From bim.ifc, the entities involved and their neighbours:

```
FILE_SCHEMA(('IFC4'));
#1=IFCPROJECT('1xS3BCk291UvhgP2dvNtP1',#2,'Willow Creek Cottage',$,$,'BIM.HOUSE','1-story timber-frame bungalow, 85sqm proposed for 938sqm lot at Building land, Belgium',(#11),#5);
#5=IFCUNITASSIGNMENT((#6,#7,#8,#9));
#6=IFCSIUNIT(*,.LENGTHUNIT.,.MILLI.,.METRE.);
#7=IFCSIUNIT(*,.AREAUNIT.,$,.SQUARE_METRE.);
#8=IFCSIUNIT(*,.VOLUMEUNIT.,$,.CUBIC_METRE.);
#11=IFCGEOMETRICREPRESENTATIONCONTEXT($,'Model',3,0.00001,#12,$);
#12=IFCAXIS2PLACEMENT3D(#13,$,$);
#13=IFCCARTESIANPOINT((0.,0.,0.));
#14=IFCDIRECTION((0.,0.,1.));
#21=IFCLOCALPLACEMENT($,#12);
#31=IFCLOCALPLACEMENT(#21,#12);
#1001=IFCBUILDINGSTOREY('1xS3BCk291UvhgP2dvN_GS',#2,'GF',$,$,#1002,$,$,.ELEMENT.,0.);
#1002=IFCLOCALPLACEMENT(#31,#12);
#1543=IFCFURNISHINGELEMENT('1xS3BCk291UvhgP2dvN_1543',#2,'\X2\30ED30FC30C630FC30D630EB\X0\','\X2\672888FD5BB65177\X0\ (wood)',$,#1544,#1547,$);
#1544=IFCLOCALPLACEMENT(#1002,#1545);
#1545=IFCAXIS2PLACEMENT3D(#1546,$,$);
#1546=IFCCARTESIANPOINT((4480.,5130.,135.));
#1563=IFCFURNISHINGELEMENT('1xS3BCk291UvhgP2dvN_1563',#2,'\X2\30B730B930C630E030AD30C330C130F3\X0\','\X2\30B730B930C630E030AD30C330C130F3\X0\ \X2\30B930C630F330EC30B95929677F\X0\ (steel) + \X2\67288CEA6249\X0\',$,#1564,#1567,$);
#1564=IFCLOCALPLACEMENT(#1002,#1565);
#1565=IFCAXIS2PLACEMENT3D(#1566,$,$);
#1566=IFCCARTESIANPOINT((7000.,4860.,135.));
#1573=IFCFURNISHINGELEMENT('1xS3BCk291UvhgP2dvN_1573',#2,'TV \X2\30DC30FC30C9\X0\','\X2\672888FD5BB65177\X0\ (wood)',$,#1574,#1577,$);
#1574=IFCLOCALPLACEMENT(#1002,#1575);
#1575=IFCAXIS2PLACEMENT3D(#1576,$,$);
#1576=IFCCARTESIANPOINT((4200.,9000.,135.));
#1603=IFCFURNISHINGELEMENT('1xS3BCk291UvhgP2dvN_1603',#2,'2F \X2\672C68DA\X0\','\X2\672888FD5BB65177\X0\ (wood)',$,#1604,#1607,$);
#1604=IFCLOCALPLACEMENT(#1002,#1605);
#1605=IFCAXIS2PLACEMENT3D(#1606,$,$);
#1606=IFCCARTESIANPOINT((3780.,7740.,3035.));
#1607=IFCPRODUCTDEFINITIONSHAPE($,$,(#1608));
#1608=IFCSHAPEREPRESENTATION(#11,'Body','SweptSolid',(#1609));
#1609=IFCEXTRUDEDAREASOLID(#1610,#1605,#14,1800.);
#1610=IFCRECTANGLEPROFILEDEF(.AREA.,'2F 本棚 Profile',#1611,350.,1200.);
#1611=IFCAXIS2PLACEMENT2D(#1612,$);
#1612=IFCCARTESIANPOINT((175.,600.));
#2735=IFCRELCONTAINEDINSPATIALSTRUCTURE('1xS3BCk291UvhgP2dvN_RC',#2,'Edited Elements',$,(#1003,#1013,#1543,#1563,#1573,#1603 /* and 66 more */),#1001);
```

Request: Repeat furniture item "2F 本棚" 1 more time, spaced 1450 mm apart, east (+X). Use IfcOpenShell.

```python
import numpy as np
import ifcopenshell
import ifcopenshell.api.geometry
import ifcopenshell.api.root
import ifcopenshell.util.element
import ifcopenshell.util.placement
import ifcopenshell.util.unit

model = ifcopenshell.open("bim.ifc")
unit_scale = ifcopenshell.util.unit.calculate_unit_scale(model)


def reuse_history(source, copy):
    """copy_class also copies each property set's owner history, people and application; keep the originals."""
    for rel in copy.IsDefinedBy:
        if rel.is_a("IfcRelDefinesByProperties") and (history := rel.RelatingPropertyDefinition.OwnerHistory):
            rel.RelatingPropertyDefinition.OwnerHistory = source.OwnerHistory
            ifcopenshell.util.element.remove_deep2(model, history)


source = model.by_id(1603)
base = ifcopenshell.util.placement.get_local_placement(source.ObjectPlacement)
step = np.array([1.0, 0.0, 0.0]) * 1.45 / unit_scale

for i in range(1, 2):
    copy = ifcopenshell.api.root.copy_class(model, product=source)
    copy.Representation = ifcopenshell.util.element.copy_deep(
        model, source.Representation, exclude=["IfcGeometricRepresentationContext", "IfcRepresentationMap"]
    )
    reuse_history(source, copy)
    matrix = base.copy()
    matrix[:3, 3] += i * step
    print("added at", matrix[:3, 3].round(3) + 0.0)
    ifcopenshell.api.geometry.edit_object_placement(model, product=copy, matrix=matrix, is_si=False)

model.write("bim_updated.ifc")
```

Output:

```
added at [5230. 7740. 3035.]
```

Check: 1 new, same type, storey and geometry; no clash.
